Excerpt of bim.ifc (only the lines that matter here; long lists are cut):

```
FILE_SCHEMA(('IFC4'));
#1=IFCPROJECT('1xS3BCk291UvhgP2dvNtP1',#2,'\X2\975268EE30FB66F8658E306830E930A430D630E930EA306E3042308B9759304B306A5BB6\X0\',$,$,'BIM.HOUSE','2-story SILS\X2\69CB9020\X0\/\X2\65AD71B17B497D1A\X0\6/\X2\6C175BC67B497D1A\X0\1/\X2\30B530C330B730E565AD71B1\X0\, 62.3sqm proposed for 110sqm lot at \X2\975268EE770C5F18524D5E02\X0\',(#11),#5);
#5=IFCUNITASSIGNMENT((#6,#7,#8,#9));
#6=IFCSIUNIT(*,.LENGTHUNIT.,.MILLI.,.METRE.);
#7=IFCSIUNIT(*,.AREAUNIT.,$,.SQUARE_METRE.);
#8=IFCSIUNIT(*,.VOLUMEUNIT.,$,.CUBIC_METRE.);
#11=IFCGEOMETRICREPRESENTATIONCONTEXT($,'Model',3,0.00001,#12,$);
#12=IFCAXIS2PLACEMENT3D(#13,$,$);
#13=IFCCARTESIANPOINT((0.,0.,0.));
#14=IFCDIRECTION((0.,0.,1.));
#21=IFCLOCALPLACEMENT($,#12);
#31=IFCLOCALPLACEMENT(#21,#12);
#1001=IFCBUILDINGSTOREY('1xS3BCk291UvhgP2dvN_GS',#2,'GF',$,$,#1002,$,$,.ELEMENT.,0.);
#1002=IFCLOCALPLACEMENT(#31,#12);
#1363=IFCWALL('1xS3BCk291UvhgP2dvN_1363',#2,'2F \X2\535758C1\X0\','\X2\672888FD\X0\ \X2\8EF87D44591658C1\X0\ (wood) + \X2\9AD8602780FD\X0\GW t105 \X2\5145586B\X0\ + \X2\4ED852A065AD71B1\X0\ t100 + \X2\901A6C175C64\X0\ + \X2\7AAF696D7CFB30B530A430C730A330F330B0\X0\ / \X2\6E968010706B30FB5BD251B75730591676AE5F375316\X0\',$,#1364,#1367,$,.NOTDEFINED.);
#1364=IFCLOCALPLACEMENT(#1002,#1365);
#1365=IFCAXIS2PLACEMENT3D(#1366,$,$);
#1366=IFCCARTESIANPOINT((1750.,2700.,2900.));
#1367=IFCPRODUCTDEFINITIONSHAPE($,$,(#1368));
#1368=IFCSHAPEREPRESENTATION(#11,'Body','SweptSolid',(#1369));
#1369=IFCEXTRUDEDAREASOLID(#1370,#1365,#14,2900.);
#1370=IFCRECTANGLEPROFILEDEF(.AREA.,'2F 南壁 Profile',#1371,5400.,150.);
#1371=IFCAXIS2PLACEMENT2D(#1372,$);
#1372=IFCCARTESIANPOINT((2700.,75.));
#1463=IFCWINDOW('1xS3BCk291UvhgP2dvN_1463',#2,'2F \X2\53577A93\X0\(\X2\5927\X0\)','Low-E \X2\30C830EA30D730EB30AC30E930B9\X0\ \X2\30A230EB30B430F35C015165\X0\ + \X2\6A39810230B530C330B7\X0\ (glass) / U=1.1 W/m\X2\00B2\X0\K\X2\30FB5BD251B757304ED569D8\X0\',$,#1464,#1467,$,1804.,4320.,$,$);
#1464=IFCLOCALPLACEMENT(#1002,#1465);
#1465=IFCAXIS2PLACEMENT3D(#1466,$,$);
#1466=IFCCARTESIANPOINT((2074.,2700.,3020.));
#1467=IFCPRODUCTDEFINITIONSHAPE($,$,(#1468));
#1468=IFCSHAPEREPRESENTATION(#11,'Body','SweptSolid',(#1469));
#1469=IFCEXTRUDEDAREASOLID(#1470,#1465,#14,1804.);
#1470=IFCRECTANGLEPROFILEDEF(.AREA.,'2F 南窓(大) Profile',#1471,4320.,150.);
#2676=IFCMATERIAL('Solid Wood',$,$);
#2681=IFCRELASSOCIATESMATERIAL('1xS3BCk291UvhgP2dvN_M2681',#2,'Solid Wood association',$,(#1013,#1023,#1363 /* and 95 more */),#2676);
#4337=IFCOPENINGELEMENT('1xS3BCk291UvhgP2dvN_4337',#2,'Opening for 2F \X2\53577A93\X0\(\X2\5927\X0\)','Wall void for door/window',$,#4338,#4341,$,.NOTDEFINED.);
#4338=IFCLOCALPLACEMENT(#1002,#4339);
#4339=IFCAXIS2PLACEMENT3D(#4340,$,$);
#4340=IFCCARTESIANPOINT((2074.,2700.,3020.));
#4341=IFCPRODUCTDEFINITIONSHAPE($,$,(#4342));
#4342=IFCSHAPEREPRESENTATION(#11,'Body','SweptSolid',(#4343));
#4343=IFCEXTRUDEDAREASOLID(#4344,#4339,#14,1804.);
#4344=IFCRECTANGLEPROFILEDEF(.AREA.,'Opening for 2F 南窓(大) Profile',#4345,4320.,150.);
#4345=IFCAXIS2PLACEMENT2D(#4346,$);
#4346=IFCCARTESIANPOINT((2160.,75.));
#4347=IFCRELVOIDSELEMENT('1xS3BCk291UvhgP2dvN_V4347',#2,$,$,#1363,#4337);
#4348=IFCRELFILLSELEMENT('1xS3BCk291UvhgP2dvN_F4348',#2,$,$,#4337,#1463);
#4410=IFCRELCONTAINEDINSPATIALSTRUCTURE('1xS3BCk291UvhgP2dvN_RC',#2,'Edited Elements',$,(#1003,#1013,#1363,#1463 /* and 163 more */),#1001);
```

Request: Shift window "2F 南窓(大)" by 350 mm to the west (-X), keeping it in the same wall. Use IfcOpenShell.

```python
import ifcopenshell
import ifcopenshell.api.geometry
import ifcopenshell.util.placement
import ifcopenshell.util.unit

model = ifcopenshell.open("bim.ifc")
unit_scale = ifcopenshell.util.unit.calculate_unit_scale(model)

window = model.by_id(1463)
opening = window.FillsVoids[0].RelatingOpeningElement
wall = opening.VoidsElements[0].RelatingBuildingElement

wall_matrix = ifcopenshell.util.placement.get_local_placement(wall.ObjectPlacement)
shift = wall_matrix[:3, 0] * -0.35 / unit_scale
before = ifcopenshell.util.placement.get_local_placement(window.ObjectPlacement)[:3, 3].copy()

# The window is not placed relative to its opening, so move both.
for product in (opening, window):
    matrix = ifcopenshell.util.placement.get_local_placement(product.ObjectPlacement)
    matrix[:3, 3] += shift
    ifcopenshell.api.geometry.edit_object_placement(model, product=product, matrix=matrix, is_si=False)

after = ifcopenshell.util.placement.get_local_placement(window.ObjectPlacement)[:3, 3]
print("window moved by", (after - before).round(3) + 0.0)

model.write("bim_edited.ifc")
```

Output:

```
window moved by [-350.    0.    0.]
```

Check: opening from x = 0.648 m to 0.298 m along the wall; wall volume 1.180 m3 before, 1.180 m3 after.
